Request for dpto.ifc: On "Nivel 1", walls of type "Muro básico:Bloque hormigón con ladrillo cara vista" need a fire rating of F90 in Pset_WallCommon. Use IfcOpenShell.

First a look at what the model holds.

```python
import ifcopenshell
import ifcopenshell.util.element

model = ifcopenshell.open("dpto.ifc")
print(model.schema)
storey = next(s for s in model.by_type("IfcBuildingStorey") if s.Name == "Nivel 1")
walls = [e for e in ifcopenshell.util.element.get_decomposition(storey) if e.is_a("IfcWall")]
seen = {}
for e in walls:
    element_type = ifcopenshell.util.element.get_type(e)
    key = (element_type.Name if element_type != e and element_type else None, ifcopenshell.util.element.get_pset(e, "Pset_WallCommon", "FireRating"))
    seen[key] = seen.get(key, 0) + 1
for (name, value), count in sorted(seen.items(), key=str):
    print(count, "x", name, "|", value)
```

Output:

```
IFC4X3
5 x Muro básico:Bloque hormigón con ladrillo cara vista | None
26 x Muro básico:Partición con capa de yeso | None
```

```python
import ifcopenshell
import ifcopenshell.api.pset
import ifcopenshell.util.element

model = ifcopenshell.open("dpto.ifc")

storey = next(s for s in model.by_type("IfcBuildingStorey") if s.Name == "Nivel 1")
walls = [e for e in ifcopenshell.util.element.get_decomposition(storey) if e.is_a("IfcWall")]

count = 0
for e in walls:
    element_type = ifcopenshell.util.element.get_type(e)
    if element_type in (None, e) or element_type.Name != "Muro básico:Bloque hormigón con ladrillo cara vista":
        continue
    # add_pset returns the element's existing set when there is one.
    pset = ifcopenshell.api.pset.add_pset(model, product=e, name="Pset_WallCommon")
    ifcopenshell.api.pset.edit_pset(model, pset=pset, properties={"FireRating": "F90"})
    count += 1

print(count, "walls updated")

model.write("dpto_updated.ifc")
```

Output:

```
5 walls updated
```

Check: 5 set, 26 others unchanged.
